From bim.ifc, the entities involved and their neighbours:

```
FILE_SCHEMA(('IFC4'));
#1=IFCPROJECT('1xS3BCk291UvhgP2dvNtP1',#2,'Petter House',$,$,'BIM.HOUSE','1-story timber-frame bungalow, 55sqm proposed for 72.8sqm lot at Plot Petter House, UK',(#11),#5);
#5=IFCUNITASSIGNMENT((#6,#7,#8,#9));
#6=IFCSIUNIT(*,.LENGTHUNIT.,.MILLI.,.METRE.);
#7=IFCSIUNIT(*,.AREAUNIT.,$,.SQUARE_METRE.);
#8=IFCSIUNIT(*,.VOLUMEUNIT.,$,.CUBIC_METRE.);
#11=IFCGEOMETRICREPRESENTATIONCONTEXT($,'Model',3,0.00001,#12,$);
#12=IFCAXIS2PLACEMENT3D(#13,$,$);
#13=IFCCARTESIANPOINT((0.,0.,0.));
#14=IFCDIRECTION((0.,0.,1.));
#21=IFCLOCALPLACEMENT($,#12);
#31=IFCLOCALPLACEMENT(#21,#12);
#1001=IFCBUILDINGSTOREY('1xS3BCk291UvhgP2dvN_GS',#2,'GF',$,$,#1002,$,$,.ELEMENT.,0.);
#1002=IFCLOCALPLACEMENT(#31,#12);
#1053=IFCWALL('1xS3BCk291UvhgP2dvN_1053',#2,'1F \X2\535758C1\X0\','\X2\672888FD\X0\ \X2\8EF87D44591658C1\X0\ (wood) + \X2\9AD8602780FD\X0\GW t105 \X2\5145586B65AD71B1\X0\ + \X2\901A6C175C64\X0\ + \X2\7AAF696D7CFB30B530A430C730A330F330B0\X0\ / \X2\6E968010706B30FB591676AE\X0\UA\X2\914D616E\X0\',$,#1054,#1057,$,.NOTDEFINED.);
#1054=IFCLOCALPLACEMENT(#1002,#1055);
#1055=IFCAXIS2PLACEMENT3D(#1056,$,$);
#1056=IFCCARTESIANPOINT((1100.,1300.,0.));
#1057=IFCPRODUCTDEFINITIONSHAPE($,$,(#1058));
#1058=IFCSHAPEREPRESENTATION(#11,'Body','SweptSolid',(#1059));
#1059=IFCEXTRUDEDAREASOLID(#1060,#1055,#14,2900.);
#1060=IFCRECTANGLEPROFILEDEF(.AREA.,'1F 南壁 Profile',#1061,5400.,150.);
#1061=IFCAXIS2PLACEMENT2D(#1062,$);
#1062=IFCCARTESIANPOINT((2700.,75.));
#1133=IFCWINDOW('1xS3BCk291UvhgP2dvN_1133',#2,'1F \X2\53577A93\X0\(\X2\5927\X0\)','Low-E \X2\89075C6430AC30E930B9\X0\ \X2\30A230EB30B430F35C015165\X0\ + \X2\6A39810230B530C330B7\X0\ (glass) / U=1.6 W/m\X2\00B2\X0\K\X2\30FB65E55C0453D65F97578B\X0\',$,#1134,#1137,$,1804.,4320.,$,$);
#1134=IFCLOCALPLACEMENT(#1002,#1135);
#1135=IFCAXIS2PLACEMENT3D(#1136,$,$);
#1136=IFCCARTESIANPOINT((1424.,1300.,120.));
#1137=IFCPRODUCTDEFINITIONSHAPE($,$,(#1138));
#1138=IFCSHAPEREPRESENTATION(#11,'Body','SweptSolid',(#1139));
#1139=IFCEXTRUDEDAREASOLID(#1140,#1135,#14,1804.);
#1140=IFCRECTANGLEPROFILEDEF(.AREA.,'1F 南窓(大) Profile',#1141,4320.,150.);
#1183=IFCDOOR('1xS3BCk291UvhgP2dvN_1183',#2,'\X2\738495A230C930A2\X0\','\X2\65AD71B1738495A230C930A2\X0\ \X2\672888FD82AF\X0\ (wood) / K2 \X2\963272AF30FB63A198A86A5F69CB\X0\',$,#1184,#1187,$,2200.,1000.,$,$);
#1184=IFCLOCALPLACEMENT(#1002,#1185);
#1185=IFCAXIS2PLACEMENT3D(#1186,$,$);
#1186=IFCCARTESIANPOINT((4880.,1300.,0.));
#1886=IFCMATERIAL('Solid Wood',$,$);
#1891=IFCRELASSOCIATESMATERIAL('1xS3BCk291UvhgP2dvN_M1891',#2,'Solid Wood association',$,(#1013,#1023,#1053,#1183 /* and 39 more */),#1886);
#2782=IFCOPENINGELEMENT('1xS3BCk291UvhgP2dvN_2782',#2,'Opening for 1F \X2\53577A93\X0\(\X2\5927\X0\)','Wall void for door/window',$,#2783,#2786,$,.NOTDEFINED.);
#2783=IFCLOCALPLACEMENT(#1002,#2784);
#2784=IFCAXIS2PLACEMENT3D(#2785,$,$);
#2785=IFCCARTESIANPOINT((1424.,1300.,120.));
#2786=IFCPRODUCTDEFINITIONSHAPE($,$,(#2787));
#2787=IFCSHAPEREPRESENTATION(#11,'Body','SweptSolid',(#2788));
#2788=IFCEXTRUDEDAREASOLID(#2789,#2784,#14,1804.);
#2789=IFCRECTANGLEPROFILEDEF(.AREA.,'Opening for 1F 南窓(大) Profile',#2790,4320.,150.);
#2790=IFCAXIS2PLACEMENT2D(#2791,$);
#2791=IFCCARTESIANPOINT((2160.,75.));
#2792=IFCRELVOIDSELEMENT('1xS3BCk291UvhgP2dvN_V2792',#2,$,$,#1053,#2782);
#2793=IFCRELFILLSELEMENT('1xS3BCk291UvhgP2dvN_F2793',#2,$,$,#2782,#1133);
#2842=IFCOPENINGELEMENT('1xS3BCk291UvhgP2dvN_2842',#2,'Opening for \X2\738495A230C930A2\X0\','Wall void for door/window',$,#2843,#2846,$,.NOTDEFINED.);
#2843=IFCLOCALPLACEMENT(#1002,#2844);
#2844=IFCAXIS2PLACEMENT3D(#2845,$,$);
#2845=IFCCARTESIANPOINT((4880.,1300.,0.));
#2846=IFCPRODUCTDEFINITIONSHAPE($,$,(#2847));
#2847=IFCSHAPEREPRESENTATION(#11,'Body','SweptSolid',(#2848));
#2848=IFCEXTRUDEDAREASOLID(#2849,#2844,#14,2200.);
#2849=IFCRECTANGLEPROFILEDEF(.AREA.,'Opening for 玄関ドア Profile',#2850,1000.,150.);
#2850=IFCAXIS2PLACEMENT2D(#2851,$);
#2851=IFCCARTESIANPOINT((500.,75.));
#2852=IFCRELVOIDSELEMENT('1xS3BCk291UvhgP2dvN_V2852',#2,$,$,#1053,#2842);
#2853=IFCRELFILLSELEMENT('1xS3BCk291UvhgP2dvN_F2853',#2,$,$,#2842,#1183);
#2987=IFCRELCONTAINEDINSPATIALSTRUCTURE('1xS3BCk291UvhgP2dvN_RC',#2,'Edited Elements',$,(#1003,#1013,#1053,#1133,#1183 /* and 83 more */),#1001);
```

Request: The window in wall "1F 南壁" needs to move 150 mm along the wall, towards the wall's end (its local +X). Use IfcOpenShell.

```python
import ifcopenshell
import ifcopenshell.api.geometry
import ifcopenshell.util.placement
import ifcopenshell.util.unit

model = ifcopenshell.open("bim.ifc")
unit_scale = ifcopenshell.util.unit.calculate_unit_scale(model)

window = model.by_guid("1xS3BCk291UvhgP2dvN_1133")
opening = window.FillsVoids[0].RelatingOpeningElement
wall = opening.VoidsElements[0].RelatingBuildingElement

wall_matrix = ifcopenshell.util.placement.get_local_placement(wall.ObjectPlacement)
shift = wall_matrix[:3, 0] * 0.15 / unit_scale
before = ifcopenshell.util.placement.get_local_placement(window.ObjectPlacement)[:3, 3].copy()

# The window is not placed relative to its opening, so move both.
for product in (opening, window):
    matrix = ifcopenshell.util.placement.get_local_placement(product.ObjectPlacement)
    matrix[:3, 3] += shift
    ifcopenshell.api.geometry.edit_object_placement(model, product=product, matrix=matrix, is_si=False)

after = ifcopenshell.util.placement.get_local_placement(window.ObjectPlacement)[:3, 3]
print("window moved by", (after - before).round(3) + 0.0)

model.write("bim-out.ifc")
```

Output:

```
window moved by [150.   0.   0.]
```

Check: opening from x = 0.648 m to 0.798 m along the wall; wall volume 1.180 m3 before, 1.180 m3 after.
